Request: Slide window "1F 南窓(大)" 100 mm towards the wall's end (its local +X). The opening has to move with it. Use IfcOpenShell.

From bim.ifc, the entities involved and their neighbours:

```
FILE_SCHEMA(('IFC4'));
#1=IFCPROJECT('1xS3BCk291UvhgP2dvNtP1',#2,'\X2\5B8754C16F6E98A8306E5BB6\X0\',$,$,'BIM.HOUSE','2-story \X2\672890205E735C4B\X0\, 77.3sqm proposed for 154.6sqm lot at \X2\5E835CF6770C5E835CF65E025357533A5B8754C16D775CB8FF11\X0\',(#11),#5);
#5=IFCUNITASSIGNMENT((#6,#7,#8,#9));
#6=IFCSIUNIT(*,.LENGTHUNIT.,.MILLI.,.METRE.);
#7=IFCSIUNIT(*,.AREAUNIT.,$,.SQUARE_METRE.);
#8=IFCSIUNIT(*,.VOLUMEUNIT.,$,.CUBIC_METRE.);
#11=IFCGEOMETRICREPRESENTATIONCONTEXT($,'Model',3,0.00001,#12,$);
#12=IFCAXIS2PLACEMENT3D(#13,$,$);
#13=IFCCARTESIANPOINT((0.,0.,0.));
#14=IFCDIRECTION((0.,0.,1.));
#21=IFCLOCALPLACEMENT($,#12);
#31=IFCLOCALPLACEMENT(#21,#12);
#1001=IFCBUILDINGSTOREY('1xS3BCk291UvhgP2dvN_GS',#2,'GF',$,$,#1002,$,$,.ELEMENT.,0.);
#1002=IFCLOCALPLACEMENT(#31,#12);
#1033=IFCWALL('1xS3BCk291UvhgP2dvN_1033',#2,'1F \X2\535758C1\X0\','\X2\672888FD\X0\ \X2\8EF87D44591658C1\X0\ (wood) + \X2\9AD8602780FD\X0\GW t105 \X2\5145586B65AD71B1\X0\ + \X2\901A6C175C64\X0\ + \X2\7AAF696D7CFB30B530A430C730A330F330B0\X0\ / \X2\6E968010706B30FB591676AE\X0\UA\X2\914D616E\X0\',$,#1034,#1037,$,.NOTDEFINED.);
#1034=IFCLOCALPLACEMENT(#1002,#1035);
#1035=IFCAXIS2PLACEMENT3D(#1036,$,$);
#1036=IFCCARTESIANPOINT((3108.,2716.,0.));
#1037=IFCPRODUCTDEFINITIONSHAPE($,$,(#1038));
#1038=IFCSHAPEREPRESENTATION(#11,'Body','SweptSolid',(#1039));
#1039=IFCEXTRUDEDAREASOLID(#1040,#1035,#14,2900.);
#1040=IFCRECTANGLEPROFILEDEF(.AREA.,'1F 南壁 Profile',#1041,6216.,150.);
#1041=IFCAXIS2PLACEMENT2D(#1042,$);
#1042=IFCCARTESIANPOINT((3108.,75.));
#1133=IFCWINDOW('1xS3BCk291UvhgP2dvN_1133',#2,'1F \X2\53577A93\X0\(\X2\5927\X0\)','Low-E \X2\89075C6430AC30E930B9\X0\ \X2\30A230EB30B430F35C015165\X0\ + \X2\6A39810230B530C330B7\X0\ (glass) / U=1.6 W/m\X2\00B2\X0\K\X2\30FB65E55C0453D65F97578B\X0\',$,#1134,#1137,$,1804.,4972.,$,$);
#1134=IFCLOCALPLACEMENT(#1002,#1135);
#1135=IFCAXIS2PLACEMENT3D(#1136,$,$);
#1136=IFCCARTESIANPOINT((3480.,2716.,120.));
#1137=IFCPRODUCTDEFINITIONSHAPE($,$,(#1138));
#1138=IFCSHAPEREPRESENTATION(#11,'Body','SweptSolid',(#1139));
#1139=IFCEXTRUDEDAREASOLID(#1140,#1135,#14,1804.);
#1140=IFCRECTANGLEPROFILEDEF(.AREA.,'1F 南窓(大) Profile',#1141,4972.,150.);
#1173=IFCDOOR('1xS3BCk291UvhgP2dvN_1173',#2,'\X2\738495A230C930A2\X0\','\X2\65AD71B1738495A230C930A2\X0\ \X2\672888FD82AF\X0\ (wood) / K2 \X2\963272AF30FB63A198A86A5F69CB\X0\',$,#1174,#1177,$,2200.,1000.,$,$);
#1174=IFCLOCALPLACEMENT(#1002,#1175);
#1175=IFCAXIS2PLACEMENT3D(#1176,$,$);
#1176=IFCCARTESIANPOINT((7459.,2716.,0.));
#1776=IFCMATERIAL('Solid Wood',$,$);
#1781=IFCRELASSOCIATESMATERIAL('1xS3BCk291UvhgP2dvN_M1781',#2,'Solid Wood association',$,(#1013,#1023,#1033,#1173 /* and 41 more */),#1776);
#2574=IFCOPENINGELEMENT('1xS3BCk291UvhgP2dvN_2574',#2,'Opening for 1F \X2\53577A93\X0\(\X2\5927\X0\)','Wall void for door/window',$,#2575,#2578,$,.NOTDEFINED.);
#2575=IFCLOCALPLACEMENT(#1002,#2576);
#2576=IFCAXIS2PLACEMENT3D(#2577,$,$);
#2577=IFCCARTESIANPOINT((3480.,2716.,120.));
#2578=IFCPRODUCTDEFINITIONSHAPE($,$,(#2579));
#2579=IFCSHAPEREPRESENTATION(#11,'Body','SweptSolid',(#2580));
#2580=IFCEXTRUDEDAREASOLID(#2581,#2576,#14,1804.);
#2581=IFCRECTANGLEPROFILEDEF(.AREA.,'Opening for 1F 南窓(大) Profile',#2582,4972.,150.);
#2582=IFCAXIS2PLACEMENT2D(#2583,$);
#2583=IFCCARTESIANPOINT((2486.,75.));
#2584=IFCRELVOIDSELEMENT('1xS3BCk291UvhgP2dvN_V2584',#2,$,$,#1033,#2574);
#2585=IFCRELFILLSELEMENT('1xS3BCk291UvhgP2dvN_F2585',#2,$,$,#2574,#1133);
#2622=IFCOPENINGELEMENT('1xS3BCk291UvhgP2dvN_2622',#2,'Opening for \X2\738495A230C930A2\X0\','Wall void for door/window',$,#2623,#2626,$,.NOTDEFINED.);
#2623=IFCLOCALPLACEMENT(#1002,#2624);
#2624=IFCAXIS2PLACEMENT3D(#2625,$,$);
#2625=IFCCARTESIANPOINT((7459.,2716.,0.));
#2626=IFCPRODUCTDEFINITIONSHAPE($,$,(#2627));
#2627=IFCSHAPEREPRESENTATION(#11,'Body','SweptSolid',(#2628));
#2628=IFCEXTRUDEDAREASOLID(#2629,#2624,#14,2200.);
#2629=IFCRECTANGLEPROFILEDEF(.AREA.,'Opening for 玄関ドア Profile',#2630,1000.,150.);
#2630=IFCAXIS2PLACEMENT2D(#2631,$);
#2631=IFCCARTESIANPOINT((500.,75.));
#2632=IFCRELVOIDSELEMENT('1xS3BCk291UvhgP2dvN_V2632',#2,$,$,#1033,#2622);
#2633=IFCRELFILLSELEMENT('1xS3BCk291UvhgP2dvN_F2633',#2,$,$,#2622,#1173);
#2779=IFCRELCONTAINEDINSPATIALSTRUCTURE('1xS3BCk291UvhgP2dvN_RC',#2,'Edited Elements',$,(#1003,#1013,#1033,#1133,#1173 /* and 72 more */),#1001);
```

```python
import ifcopenshell
import ifcopenshell.api.geometry
import ifcopenshell.util.placement
import ifcopenshell.util.unit

model = ifcopenshell.open("bim.ifc")
unit_scale = ifcopenshell.util.unit.calculate_unit_scale(model)

window = model.by_id(1133)
opening = window.FillsVoids[0].RelatingOpeningElement
wall = opening.VoidsElements[0].RelatingBuildingElement

wall_matrix = ifcopenshell.util.placement.get_local_placement(wall.ObjectPlacement)
shift = wall_matrix[:3, 0] * 0.1 / unit_scale
before = ifcopenshell.util.placement.get_local_placement(window.ObjectPlacement)[:3, 3].copy()

# The window is not placed relative to its opening, so move both.
for product in (opening, window):
    matrix = ifcopenshell.util.placement.get_local_placement(product.ObjectPlacement)
    matrix[:3, 3] += shift
    ifcopenshell.api.geometry.edit_object_placement(model, product=product, matrix=matrix, is_si=False)

after = ifcopenshell.util.placement.get_local_placement(window.ObjectPlacement)[:3, 3]
print("window moved by", (after - before).round(3) + 0.0)

model.write("bim_rev.ifc")
```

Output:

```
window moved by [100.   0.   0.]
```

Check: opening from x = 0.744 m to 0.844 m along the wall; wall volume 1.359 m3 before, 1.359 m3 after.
